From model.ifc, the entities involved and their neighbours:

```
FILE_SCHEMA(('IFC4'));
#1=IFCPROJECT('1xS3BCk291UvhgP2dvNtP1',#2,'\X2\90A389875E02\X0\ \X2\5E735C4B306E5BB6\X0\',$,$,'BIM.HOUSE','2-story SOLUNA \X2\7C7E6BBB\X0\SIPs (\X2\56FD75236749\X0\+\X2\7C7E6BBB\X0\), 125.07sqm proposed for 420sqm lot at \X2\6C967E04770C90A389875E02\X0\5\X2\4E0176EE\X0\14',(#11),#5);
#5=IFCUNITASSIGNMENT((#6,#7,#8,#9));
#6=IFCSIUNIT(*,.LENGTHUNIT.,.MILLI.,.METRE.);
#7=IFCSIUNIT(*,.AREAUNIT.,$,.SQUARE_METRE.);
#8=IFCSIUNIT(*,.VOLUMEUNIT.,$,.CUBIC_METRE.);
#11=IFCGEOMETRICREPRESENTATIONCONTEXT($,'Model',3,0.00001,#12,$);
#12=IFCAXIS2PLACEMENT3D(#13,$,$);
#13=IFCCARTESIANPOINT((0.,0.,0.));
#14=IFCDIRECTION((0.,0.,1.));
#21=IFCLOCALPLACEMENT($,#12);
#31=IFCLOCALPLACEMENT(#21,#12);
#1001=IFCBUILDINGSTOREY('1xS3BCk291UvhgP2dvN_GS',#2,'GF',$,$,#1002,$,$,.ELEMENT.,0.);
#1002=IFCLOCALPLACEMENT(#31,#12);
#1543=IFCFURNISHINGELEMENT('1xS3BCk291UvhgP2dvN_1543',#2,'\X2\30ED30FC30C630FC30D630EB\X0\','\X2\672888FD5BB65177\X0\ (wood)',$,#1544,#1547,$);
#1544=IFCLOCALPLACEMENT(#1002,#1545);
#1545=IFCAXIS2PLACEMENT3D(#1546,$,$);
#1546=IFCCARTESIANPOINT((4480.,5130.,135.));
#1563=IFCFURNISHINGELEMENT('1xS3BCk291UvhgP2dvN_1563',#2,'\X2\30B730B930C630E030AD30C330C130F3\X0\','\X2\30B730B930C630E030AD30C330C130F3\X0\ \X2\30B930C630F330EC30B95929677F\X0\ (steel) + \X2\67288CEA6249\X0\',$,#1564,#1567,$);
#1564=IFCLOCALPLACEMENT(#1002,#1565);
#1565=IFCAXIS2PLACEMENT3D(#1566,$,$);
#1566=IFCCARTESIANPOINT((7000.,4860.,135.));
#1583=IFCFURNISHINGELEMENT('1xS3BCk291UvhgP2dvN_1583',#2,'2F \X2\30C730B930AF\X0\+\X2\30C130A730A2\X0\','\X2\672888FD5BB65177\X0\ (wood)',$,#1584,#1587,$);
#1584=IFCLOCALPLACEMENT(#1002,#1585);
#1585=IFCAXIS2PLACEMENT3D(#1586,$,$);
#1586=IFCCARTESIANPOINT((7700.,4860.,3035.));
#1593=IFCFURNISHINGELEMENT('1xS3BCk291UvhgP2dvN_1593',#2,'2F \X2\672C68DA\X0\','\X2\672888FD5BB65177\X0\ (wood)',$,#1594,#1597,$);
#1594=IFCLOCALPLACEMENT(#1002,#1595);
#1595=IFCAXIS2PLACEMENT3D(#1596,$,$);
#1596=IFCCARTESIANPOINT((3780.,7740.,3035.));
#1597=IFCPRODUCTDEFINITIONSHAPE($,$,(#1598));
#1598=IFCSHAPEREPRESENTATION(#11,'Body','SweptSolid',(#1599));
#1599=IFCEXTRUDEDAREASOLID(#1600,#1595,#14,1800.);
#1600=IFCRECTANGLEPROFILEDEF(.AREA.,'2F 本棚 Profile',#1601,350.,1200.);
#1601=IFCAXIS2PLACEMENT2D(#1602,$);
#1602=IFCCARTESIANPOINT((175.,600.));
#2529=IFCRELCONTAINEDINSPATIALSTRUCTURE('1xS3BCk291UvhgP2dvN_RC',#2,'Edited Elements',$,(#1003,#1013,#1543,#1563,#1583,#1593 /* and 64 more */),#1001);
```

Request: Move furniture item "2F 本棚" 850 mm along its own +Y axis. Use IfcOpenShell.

```python
import ifcopenshell
import ifcopenshell.api.geometry
import ifcopenshell.util.placement

model = ifcopenshell.open("model.ifc")

item = model.by_id(1593)
matrix = ifcopenshell.util.placement.get_local_placement(item.ObjectPlacement)
matrix[:3, 3] += matrix[:3, 1] * 850.0
ifcopenshell.api.geometry.edit_object_placement(model, product=item, matrix=matrix, is_si=False)

print(ifcopenshell.util.placement.get_local_placement(item.ObjectPlacement).round(3) + 0.0)

model.write("model_updated.ifc")
```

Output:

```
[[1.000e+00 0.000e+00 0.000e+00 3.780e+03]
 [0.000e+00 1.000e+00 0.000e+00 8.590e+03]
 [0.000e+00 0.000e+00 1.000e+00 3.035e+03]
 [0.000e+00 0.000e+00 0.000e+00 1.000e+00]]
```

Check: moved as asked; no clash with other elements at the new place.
